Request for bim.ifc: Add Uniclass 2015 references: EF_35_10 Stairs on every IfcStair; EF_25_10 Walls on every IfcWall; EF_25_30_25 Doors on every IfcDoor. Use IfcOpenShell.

First a look at what the model holds.

```python
import ifcopenshell

model = ifcopenshell.open("bim.ifc")
print(model.schema)
print("classifications:", [c.Name for c in model.by_type("IfcClassification")])
for ifc_class in ("IfcDoor", "IfcRoof", "IfcStair", "IfcWall", "IfcWindow"):
    print(ifc_class, len(model.by_type(ifc_class)))
```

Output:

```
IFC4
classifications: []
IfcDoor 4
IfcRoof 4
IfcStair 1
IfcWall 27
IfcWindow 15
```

```python
import ifcopenshell
import ifcopenshell.api.classification

model = ifcopenshell.open("bim.ifc")

system = ifcopenshell.api.classification.add_classification(model, classification="Uniclass 2015")

codes = {
    "IfcStair": ("EF_35_10", "Stairs"),
    "IfcWall": ("EF_25_10", "Walls"),
    "IfcDoor": ("EF_25_30_25", "Doors"),
}
for ifc_class, (code, name) in codes.items():
    products = model.by_type(ifc_class)
    ifcopenshell.api.classification.add_reference(
        model, products=products, classification=system, identification=code, name=name
    )
    print(code, len(products))

model.write("bim_v2.ifc")
```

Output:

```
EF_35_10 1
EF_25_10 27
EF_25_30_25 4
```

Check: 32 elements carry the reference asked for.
